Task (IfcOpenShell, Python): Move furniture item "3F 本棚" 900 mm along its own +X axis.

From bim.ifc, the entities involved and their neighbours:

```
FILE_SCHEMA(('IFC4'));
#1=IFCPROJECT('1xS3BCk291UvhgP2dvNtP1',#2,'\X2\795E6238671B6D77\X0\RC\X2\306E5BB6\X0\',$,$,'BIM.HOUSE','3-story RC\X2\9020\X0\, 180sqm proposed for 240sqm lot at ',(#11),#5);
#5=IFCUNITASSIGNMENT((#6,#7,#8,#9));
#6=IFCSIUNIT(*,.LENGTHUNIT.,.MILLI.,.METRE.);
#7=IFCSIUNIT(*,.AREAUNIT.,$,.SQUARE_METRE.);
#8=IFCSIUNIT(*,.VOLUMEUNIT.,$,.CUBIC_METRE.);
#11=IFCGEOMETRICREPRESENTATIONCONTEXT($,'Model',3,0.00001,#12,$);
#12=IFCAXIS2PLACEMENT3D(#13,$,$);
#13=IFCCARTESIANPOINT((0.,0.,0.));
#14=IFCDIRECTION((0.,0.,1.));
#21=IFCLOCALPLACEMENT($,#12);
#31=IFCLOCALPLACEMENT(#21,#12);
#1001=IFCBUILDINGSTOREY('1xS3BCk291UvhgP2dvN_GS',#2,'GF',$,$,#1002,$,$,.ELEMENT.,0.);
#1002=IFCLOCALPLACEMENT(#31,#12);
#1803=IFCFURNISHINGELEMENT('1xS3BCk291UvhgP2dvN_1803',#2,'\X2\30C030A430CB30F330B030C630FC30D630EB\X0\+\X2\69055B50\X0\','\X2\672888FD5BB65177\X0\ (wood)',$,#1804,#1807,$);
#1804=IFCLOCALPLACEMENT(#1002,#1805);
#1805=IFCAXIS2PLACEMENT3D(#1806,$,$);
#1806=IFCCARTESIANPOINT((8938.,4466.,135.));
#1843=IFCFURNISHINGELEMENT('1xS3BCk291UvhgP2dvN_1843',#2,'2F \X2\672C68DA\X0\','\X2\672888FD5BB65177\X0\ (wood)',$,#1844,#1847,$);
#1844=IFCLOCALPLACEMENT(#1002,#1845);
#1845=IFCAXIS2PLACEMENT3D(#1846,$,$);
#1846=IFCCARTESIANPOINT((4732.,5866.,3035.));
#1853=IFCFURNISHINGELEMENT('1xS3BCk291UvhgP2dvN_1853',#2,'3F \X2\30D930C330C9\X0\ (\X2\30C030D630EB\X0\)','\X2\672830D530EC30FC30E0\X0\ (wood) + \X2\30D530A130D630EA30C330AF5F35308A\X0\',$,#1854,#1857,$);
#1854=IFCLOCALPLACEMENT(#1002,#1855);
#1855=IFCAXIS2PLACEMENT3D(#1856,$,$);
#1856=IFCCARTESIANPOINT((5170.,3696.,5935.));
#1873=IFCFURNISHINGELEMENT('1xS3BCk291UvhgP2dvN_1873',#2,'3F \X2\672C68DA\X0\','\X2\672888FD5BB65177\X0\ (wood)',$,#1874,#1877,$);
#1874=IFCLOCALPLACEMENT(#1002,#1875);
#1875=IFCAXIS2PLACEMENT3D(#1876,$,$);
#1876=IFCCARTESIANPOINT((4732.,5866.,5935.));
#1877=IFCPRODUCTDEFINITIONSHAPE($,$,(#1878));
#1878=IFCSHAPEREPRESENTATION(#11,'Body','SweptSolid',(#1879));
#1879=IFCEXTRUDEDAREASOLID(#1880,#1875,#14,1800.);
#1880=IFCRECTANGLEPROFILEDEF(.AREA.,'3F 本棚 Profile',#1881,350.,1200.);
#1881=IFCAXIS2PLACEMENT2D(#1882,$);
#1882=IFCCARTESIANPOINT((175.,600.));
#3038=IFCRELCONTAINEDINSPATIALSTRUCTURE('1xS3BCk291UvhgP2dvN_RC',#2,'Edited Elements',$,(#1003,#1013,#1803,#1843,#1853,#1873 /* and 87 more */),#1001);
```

```python
import ifcopenshell
import ifcopenshell.api.geometry
import ifcopenshell.util.placement

model = ifcopenshell.open("bim.ifc")

item = model.by_guid("1xS3BCk291UvhgP2dvN_1873")
matrix = ifcopenshell.util.placement.get_local_placement(item.ObjectPlacement)
matrix[:3, 3] += matrix[:3, 0] * 900.0
ifcopenshell.api.geometry.edit_object_placement(model, product=item, matrix=matrix, is_si=False)

print(ifcopenshell.util.placement.get_local_placement(item.ObjectPlacement).round(3) + 0.0)

model.write("bim_v2.ifc")
```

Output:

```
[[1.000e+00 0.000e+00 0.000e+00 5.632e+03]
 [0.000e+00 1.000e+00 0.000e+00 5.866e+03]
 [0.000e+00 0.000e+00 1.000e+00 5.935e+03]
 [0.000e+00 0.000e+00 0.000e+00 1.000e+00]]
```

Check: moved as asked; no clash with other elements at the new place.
